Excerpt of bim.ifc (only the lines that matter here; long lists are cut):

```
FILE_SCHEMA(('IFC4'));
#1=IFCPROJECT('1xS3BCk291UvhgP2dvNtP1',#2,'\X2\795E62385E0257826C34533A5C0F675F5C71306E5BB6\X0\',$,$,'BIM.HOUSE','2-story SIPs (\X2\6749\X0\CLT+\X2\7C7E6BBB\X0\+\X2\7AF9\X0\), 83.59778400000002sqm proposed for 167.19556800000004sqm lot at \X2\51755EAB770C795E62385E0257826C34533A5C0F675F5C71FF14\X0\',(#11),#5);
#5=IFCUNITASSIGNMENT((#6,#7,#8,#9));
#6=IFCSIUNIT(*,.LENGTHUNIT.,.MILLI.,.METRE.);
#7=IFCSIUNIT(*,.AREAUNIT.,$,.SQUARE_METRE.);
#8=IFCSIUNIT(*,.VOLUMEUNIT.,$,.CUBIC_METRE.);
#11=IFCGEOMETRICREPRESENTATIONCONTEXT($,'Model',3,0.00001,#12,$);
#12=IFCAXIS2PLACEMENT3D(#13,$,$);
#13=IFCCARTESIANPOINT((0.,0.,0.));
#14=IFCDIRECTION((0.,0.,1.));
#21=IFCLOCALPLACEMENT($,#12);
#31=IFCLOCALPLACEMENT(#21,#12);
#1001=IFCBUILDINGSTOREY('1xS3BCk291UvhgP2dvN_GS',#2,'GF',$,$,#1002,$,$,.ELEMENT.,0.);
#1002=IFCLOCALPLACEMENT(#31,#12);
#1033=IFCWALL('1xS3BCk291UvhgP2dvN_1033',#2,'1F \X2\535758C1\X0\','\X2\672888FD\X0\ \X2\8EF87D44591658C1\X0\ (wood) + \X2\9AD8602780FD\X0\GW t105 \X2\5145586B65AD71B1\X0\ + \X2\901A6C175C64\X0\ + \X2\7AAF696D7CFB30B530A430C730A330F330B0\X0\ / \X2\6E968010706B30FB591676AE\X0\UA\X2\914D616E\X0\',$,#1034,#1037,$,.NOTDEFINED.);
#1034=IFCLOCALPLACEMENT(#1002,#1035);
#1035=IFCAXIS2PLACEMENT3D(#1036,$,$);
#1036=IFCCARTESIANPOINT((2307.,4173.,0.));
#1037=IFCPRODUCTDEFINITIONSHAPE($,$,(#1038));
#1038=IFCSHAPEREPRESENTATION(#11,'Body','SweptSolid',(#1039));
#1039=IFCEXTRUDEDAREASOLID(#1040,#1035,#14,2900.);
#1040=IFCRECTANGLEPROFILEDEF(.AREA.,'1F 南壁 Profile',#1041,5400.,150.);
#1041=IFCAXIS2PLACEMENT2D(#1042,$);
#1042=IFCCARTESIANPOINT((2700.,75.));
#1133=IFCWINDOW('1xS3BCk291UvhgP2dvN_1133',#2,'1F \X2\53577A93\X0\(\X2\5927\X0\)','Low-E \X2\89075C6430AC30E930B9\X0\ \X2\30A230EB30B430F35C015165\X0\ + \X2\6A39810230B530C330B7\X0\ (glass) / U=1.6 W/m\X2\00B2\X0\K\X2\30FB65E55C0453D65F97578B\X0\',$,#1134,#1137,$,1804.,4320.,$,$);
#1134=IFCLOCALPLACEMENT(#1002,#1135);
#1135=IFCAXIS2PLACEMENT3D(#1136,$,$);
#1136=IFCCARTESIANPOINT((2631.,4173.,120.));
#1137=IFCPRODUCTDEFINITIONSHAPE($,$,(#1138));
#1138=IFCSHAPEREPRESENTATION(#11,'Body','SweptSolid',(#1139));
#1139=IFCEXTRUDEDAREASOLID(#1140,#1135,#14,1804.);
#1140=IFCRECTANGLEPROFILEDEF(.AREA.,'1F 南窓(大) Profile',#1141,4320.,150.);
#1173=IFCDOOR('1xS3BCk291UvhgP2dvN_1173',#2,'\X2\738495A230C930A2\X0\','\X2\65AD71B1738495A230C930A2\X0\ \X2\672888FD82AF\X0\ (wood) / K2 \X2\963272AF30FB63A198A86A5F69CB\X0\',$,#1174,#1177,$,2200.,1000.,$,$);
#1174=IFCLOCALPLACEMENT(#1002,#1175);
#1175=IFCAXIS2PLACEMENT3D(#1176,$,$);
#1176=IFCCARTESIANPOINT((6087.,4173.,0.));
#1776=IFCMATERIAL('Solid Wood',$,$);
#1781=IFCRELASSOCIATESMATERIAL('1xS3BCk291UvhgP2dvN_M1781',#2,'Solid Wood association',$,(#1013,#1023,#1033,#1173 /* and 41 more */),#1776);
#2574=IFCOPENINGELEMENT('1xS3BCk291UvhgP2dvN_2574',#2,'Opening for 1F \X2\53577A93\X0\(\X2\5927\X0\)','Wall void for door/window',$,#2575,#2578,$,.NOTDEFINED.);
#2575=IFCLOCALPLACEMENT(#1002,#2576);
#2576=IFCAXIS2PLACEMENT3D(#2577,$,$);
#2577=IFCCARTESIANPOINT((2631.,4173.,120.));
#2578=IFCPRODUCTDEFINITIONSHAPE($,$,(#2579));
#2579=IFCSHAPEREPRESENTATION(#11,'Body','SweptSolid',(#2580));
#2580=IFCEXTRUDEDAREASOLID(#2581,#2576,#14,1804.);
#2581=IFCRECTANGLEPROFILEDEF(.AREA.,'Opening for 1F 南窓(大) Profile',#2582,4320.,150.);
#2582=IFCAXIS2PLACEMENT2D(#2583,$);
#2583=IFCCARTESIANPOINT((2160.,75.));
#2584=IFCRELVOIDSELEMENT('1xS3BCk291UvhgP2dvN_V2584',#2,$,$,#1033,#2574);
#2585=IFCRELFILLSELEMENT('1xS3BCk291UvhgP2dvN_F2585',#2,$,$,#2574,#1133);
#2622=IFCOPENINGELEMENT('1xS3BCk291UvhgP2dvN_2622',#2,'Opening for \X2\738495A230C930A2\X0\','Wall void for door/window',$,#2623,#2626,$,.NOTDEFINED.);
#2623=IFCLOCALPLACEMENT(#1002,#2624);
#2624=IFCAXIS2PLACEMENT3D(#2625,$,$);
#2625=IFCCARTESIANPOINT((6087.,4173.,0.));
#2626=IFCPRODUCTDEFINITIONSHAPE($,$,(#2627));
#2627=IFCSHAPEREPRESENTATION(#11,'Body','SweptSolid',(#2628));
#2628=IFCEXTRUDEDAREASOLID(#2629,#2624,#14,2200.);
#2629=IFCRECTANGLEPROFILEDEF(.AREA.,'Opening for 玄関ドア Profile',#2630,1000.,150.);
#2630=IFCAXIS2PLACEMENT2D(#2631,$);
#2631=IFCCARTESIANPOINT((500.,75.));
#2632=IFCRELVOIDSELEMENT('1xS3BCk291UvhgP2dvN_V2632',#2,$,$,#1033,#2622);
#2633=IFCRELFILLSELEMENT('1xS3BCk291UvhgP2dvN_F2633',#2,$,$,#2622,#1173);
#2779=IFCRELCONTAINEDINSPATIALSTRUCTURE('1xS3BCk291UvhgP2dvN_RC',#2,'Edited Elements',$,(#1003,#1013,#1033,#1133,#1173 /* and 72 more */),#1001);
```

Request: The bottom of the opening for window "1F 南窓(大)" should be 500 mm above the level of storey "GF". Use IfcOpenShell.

```python
import numpy as np
import ifcopenshell
import ifcopenshell.api.geometry
import ifcopenshell.geom
import ifcopenshell.util.element
import ifcopenshell.util.placement
import ifcopenshell.util.shape
import ifcopenshell.util.unit

model = ifcopenshell.open("bim.ifc")
unit_scale = ifcopenshell.util.unit.calculate_unit_scale(model)

window = model.by_guid("1xS3BCk291UvhgP2dvN_1133")
opening = window.FillsVoids[0].RelatingOpeningElement
storey = ifcopenshell.util.element.get_container(window, ifc_class="IfcBuildingStorey")
level = ifcopenshell.util.placement.get_local_placement(storey.ObjectPlacement)[2, 3]

# The opening's origin need not be at the sill, so measure its lowest point.
shape = ifcopenshell.geom.create_shape(ifcopenshell.geom.settings(), opening)
bottom = ifcopenshell.util.shape.get_shape_bottom_elevation(shape, shape.geometry) / unit_scale
dz = level + 0.5 / unit_scale - bottom

shift = np.array([0.0, 0.0, dz])
# The window is not placed relative to its opening, so move both.
for product in (opening, window):
    matrix = ifcopenshell.util.placement.get_local_placement(product.ObjectPlacement)
    matrix[:3, 3] += shift
    ifcopenshell.api.geometry.edit_object_placement(model, product=product, matrix=matrix, is_si=False)

print(f"moved by {dz * unit_scale:+.3f} m")

model.write("bim_edited.ifc")
```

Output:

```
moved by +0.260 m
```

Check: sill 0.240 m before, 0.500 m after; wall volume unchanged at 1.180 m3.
